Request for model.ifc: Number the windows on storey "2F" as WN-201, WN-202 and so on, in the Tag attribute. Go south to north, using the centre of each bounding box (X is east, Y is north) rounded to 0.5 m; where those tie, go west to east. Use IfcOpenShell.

First a look at what the model holds.

```python
import ifcopenshell
import ifcopenshell.util.element
import ifcopenshell.util.placement

model = ifcopenshell.open("model.ifc")
print(model.schema)
storey = next(s for s in model.by_type("IfcBuildingStorey") if s.Name == "2F")
windows = [e for e in ifcopenshell.util.element.get_decomposition(storey) if e.is_a("IfcWindow")]
for e in sorted(windows, key=lambda e: e.id()):
    origin = ifcopenshell.util.placement.get_local_placement(e.ObjectPlacement)[:3, 3]
    print(e.id(), e.Tag, e.Name, origin.round(2) + 0.0, sep=" | ")
```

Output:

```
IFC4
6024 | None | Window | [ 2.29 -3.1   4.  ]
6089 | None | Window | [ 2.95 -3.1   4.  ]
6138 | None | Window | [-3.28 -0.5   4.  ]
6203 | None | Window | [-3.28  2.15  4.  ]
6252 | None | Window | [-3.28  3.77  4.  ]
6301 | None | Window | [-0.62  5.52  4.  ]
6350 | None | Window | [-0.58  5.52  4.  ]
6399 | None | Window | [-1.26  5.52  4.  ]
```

```python
import ifcopenshell
import ifcopenshell.geom
import ifcopenshell.util.element
import ifcopenshell.util.shape

model = ifcopenshell.open("model.ifc")
settings = ifcopenshell.geom.settings()
settings.set("use-world-coords", True)


def centre(element):
    shape = ifcopenshell.geom.create_shape(settings, element)
    return ifcopenshell.util.shape.get_bbox_centroid(shape.geometry)


storey = next(s for s in model.by_type("IfcBuildingStorey") if s.Name == "2F")
windows = [e for e in ifcopenshell.util.element.get_decomposition(storey) if e.is_a("IfcWindow")]

# Insertion points can sit at a corner or the storey origin, so sort by the geometry (in metres).
centres = {e: centre(e) for e in windows}
windows.sort(key=lambda e: (round(centres[e][1] / 0.5), centres[e][0]))

for i, e in enumerate(windows, start=1):
    number = f"WN-2{i:02d}"
    e.Tag = number
    print(e.id(), number)

model.write("model_v2.ifc")
```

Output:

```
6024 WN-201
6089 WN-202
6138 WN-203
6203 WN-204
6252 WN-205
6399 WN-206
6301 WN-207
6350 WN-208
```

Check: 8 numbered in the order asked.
